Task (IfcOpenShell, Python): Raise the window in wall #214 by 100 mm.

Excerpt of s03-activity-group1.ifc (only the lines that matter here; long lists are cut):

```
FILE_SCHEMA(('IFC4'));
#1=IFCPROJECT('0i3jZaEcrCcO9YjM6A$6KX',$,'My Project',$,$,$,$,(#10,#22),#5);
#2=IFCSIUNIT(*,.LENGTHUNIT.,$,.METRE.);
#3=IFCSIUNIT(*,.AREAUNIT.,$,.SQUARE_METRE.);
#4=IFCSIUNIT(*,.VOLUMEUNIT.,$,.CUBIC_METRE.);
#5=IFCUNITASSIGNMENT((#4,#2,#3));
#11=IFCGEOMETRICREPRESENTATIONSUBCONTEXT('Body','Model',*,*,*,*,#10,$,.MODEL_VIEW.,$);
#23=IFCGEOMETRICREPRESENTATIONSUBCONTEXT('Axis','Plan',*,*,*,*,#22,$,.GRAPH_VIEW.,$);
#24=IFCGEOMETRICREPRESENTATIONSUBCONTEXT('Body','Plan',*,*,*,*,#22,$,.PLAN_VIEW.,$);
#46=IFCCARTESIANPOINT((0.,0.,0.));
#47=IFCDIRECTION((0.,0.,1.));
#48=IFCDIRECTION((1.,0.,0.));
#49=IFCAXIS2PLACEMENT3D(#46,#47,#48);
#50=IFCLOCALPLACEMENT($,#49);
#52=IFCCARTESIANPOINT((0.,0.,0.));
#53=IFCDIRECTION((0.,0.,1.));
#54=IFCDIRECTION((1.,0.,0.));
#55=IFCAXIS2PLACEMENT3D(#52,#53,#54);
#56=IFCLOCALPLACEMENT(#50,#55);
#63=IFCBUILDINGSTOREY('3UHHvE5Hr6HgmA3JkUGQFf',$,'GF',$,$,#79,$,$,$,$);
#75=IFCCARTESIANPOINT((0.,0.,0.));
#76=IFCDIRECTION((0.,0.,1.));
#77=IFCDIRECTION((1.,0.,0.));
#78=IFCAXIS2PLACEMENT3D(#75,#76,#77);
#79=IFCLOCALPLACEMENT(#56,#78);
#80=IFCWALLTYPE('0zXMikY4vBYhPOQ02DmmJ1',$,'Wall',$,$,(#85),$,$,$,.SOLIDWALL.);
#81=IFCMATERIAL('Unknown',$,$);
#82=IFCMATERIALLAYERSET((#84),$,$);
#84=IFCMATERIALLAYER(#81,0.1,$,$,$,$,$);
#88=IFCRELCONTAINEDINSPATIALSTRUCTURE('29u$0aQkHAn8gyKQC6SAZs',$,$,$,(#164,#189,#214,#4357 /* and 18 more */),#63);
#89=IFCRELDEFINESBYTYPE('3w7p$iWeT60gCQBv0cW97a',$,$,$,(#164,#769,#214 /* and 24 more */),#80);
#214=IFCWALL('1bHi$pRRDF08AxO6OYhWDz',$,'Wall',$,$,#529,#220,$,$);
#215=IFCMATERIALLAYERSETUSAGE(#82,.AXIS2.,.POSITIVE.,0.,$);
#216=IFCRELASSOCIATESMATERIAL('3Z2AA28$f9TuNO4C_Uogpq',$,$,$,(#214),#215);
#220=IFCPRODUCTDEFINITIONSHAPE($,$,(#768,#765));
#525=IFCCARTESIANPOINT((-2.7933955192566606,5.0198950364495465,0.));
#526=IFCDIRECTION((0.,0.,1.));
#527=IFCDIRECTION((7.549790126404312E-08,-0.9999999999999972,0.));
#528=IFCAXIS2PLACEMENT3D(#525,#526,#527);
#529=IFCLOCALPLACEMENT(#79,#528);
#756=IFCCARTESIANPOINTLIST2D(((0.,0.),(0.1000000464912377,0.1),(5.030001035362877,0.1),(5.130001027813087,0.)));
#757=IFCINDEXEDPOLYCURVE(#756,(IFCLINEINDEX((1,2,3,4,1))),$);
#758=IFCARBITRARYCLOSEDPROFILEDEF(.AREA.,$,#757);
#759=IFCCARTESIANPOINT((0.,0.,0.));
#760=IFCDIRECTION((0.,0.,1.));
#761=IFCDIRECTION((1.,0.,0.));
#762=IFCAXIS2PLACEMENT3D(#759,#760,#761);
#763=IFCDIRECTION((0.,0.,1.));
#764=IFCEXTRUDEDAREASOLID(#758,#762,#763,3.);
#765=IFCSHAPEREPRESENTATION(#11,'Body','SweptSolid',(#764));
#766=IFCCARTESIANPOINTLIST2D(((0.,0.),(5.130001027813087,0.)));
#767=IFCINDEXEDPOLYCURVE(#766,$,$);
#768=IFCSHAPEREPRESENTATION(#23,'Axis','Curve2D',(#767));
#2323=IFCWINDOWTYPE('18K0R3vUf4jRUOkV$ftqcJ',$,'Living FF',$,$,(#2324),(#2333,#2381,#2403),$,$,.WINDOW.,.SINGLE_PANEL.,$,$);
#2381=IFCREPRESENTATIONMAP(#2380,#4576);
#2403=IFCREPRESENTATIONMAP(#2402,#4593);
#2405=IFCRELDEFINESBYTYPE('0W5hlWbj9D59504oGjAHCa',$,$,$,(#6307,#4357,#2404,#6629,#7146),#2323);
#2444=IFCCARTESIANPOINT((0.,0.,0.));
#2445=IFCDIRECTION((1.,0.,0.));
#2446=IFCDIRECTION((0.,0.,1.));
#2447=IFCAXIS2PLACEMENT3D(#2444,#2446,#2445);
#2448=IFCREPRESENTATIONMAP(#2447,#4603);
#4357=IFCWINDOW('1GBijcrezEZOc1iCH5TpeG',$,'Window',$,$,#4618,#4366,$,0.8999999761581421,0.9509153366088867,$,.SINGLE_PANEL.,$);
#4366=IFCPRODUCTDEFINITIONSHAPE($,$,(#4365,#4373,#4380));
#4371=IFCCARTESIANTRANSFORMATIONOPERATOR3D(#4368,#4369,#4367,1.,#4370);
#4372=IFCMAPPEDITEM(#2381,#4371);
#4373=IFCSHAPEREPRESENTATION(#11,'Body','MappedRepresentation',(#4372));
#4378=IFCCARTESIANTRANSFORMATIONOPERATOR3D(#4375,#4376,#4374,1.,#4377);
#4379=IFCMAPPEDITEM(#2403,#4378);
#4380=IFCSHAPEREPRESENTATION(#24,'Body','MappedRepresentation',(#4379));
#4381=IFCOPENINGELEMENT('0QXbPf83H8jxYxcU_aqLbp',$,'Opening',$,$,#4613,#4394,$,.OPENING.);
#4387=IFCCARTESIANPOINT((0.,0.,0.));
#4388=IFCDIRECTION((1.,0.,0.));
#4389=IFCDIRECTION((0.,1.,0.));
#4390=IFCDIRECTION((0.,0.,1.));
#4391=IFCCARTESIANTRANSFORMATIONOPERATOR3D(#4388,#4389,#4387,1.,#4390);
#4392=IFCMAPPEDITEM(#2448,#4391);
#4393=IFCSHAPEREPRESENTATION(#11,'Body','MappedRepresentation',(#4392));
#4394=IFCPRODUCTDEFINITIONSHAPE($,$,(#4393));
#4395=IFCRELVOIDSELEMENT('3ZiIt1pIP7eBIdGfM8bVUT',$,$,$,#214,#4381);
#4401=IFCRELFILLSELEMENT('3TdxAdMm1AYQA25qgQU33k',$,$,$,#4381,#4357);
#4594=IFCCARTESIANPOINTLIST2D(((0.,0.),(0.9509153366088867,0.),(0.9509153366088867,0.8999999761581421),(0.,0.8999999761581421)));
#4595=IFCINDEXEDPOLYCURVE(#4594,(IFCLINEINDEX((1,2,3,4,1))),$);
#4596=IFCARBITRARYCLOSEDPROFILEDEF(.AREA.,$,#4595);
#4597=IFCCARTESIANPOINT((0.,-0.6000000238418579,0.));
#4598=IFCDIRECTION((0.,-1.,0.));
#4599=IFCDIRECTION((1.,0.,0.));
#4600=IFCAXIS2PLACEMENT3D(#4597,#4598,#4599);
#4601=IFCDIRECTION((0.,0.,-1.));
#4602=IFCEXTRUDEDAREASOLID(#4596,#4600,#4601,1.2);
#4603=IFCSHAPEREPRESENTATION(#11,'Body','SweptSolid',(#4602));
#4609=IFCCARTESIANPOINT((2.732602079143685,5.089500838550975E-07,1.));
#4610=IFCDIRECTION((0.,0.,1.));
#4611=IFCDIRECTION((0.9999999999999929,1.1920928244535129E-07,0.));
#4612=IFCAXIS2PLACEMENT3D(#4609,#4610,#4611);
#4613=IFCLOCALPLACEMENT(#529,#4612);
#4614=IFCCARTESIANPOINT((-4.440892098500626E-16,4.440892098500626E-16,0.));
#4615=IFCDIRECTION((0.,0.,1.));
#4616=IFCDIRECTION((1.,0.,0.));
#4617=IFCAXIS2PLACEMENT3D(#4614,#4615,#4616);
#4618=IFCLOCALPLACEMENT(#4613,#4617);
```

```python
import numpy as np
import ifcopenshell
import ifcopenshell.api.geometry
import ifcopenshell.util.placement
import ifcopenshell.util.unit

model = ifcopenshell.open("s03-activity-group1.ifc")
unit_scale = ifcopenshell.util.unit.calculate_unit_scale(model)

window = model.by_guid("1GBijcrezEZOc1iCH5TpeG")
opening = window.FillsVoids[0].RelatingOpeningElement
dz = 0.1 / unit_scale

shift = np.array([0.0, 0.0, dz])
# The window is placed relative to its opening, so it follows when the opening moves.
matrix = ifcopenshell.util.placement.get_local_placement(opening.ObjectPlacement)
matrix[:3, 3] += shift
ifcopenshell.api.geometry.edit_object_placement(
    model, product=opening, matrix=matrix, is_si=False, should_transform_children=True
)

print(f"moved by {dz * unit_scale:+.3f} m")

model.write("s03-activity-group1_rev.ifc")
```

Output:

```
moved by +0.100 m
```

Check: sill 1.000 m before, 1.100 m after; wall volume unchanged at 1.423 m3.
